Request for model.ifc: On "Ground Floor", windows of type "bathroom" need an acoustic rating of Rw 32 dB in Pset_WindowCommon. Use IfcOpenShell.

First a look at what the model holds.

```python
import ifcopenshell
import ifcopenshell.util.element

model = ifcopenshell.open("model.ifc")
print(model.schema)
storey = next(s for s in model.by_type("IfcBuildingStorey") if s.Name == "Ground Floor")
windows = [e for e in ifcopenshell.util.element.get_decomposition(storey) if e.is_a("IfcWindow")]
seen = {}
for e in windows:
    element_type = ifcopenshell.util.element.get_type(e)
    key = (element_type.Name if element_type != e and element_type else None, ifcopenshell.util.element.get_pset(e, "Pset_WindowCommon", "AcousticRating"))
    seen[key] = seen.get(key, 0) + 1
for (name, value), count in sorted(seen.items(), key=str):
    print(count, "x", name, "|", value)
```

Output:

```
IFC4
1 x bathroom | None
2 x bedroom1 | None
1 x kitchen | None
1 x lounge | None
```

```python
import ifcopenshell
import ifcopenshell.api.pset
import ifcopenshell.util.element

model = ifcopenshell.open("model.ifc")

storey = next(s for s in model.by_type("IfcBuildingStorey") if s.Name == "Ground Floor")
windows = [e for e in ifcopenshell.util.element.get_decomposition(storey) if e.is_a("IfcWindow")]

count = 0
for e in windows:
    element_type = ifcopenshell.util.element.get_type(e)
    if element_type in (None, e) or element_type.Name != "bathroom":
        continue
    # add_pset returns the element's existing set when there is one.
    pset = ifcopenshell.api.pset.add_pset(model, product=e, name="Pset_WindowCommon")
    ifcopenshell.api.pset.edit_pset(model, pset=pset, properties={"AcousticRating": "Rw 32 dB"})
    count += 1

print(count, "windows updated")

model.write("model_edited.ifc")
```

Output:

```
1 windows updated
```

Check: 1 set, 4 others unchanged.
